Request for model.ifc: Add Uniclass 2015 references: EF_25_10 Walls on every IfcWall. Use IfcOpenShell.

First a look at what the model holds.

```python
import ifcopenshell

model = ifcopenshell.open("model.ifc")
print(model.schema)
print("classifications:", [c.Name for c in model.by_type("IfcClassification")])
for ifc_class in ("IfcDoor", "IfcRoof", "IfcStair", "IfcWall", "IfcWindow"):
    print(ifc_class, len(model.by_type(ifc_class)))
```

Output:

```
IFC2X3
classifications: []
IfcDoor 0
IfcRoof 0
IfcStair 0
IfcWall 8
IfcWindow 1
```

```python
import ifcopenshell
import ifcopenshell.api.classification

model = ifcopenshell.open("model.ifc")

# IFC2X3 requires Source and Edition and has no link from the project to the system.
system = model.create_entity("IfcClassification", Source="NBS", Edition="2015", Name="Uniclass 2015")

codes = {
    "IfcWall": ("EF_25_10", "Walls"),
}
for ifc_class, (code, name) in codes.items():
    products = model.by_type(ifc_class)
    ifcopenshell.api.classification.add_reference(
        model, products=products, classification=system, identification=code, name=name
    )
    print(code, len(products))

model.write("model_v2.ifc")
```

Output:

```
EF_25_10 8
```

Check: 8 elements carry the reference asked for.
